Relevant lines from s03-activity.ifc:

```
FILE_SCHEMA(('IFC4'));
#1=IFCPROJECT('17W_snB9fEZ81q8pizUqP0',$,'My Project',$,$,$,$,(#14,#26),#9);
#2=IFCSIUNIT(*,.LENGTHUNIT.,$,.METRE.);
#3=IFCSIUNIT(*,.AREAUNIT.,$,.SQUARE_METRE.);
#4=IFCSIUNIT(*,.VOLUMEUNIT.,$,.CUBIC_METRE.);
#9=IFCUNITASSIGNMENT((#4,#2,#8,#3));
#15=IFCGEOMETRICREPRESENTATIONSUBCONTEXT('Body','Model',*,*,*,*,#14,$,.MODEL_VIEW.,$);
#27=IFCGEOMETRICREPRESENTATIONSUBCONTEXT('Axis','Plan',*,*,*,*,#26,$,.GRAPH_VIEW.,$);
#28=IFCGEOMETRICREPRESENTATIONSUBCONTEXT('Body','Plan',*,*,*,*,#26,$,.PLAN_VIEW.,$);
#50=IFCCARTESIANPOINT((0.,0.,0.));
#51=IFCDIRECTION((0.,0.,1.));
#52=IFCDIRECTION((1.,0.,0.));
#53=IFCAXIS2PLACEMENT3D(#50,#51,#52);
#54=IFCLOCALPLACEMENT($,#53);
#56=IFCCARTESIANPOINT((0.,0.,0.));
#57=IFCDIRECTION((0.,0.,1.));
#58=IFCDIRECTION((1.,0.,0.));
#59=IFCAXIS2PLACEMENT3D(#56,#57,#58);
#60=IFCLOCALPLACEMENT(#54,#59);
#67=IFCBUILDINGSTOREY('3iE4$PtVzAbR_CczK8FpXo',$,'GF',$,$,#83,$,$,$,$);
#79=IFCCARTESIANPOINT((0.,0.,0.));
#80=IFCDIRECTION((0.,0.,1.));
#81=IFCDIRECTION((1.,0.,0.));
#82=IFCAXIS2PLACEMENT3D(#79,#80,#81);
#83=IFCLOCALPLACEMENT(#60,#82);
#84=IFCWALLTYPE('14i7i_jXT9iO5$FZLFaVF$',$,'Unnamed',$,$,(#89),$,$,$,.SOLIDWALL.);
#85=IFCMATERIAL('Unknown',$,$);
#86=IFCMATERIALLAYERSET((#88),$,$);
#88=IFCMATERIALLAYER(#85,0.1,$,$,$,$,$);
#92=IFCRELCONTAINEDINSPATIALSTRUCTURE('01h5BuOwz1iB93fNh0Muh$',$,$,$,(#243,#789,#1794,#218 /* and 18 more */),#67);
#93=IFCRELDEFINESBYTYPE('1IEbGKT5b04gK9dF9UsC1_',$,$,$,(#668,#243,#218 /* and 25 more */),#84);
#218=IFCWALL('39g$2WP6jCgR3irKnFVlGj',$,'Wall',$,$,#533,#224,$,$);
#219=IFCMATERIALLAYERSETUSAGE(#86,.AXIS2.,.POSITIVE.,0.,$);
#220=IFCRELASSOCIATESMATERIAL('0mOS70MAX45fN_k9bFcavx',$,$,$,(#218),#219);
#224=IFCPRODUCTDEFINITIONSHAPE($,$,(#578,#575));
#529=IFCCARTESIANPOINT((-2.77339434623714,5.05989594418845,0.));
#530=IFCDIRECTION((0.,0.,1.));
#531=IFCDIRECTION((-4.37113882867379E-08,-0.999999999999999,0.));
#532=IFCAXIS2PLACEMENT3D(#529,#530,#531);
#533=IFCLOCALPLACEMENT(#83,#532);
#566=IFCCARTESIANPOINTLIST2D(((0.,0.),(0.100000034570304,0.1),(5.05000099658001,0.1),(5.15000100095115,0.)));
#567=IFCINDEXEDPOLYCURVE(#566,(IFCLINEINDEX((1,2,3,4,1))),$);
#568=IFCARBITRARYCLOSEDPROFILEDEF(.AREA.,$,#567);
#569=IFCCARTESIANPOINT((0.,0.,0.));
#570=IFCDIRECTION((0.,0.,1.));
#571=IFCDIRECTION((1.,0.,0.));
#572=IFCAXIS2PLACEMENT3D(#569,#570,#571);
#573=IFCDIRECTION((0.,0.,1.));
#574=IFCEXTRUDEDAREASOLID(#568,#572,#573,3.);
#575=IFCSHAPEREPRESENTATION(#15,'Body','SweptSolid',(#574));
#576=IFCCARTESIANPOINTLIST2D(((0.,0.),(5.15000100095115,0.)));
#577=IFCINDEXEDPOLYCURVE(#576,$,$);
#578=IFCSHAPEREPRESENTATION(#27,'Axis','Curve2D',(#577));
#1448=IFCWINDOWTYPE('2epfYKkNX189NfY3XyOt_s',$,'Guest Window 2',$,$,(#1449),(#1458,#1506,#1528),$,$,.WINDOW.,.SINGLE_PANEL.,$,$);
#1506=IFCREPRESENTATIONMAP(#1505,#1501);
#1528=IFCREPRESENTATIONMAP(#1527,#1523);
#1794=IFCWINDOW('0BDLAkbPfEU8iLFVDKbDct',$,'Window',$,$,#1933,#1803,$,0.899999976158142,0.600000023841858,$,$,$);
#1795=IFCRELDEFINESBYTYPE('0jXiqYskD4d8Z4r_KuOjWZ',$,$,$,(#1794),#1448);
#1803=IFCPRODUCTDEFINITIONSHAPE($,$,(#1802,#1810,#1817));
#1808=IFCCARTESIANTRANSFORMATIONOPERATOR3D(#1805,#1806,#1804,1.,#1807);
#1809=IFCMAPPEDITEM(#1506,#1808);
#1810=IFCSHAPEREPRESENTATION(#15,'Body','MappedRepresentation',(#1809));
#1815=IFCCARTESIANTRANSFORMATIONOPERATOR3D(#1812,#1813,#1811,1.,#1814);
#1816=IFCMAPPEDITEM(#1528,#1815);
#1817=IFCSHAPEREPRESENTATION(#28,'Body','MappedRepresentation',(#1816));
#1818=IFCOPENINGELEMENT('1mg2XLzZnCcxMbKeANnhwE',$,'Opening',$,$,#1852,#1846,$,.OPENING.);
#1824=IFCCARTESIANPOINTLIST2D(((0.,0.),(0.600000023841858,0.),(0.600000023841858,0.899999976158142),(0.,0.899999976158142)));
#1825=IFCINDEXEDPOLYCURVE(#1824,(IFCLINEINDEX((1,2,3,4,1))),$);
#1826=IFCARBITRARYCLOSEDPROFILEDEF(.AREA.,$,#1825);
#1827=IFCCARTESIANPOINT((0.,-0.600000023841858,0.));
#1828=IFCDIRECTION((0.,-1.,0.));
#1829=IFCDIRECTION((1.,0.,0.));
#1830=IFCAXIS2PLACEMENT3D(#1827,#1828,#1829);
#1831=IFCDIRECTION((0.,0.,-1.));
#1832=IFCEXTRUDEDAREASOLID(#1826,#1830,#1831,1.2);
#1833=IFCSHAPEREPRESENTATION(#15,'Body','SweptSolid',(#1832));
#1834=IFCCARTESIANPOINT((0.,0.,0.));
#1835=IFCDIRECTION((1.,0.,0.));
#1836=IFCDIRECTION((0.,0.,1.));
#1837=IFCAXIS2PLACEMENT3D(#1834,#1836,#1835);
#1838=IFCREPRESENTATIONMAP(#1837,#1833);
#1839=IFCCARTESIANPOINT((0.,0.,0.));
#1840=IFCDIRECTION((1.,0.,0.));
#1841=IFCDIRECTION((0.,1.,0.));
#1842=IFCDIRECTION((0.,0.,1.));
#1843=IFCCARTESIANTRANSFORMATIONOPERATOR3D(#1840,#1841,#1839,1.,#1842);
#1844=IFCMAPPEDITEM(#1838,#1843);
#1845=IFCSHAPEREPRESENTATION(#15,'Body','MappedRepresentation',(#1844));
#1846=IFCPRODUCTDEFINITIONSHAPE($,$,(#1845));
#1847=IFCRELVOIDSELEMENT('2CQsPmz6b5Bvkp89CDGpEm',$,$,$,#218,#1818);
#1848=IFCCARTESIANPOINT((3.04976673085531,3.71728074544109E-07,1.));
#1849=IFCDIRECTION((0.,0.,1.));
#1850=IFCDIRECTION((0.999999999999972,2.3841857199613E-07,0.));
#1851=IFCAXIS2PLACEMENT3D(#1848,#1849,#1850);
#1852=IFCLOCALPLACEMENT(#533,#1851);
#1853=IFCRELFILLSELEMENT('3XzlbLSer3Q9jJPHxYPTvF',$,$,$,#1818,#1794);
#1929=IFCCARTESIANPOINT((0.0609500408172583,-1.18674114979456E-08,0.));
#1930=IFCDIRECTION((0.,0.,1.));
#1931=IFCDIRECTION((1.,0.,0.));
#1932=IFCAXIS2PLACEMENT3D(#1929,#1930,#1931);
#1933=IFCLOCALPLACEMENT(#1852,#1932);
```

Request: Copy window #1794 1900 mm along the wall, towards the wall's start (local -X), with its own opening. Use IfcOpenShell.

```python
import ifcopenshell
import ifcopenshell.api.feature
import ifcopenshell.api.geometry
import ifcopenshell.api.root
import ifcopenshell.geom
import ifcopenshell.util.element
import ifcopenshell.util.placement
import ifcopenshell.util.shape

model = ifcopenshell.open("s03-activity.ifc")
settings = ifcopenshell.geom.settings()


def volume(element):
    """Net volume in cubic metres, openings subtracted."""
    shape = ifcopenshell.geom.create_shape(settings, element)
    return ifcopenshell.util.shape.get_volume(shape.geometry)


window = model.by_guid("0BDLAkbPfEU8iLFVDKbDct")
opening = window.FillsVoids[0].RelatingOpeningElement
wall = opening.VoidsElements[0].RelatingBuildingElement
before = volume(wall)
shift = ifcopenshell.util.placement.get_local_placement(wall.ObjectPlacement)[:3, 0] * -1.9

# copy_class copies the void relationship, type, container and properties, but no geometry.
new_opening = ifcopenshell.api.root.copy_class(model, product=opening)
new_opening.Representation = ifcopenshell.util.element.copy_deep(
    model, opening.Representation, exclude=["IfcGeometricRepresentationContext", "IfcRepresentationMap"]
)
new_window = ifcopenshell.api.root.copy_class(model, product=window)
new_window.Representation = ifcopenshell.util.element.copy_deep(
    model, window.Representation, exclude=["IfcGeometricRepresentationContext", "IfcRepresentationMap"]
)
ifcopenshell.api.feature.add_filling(model, opening=new_opening, element=new_window)

for old, new in ((opening, new_opening), (window, new_window)):
    matrix = ifcopenshell.util.placement.get_local_placement(old.ObjectPlacement)
    matrix[:3, 3] += shift
    ifcopenshell.api.geometry.edit_object_placement(model, product=new, matrix=matrix, is_si=False)

after = volume(wall)

print(f"wall volume {before:.3f} -> {after:.3f} m3")

model.write("s03-activity-out.ifc")
```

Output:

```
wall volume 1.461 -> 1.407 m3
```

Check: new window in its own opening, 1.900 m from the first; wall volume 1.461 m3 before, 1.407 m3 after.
